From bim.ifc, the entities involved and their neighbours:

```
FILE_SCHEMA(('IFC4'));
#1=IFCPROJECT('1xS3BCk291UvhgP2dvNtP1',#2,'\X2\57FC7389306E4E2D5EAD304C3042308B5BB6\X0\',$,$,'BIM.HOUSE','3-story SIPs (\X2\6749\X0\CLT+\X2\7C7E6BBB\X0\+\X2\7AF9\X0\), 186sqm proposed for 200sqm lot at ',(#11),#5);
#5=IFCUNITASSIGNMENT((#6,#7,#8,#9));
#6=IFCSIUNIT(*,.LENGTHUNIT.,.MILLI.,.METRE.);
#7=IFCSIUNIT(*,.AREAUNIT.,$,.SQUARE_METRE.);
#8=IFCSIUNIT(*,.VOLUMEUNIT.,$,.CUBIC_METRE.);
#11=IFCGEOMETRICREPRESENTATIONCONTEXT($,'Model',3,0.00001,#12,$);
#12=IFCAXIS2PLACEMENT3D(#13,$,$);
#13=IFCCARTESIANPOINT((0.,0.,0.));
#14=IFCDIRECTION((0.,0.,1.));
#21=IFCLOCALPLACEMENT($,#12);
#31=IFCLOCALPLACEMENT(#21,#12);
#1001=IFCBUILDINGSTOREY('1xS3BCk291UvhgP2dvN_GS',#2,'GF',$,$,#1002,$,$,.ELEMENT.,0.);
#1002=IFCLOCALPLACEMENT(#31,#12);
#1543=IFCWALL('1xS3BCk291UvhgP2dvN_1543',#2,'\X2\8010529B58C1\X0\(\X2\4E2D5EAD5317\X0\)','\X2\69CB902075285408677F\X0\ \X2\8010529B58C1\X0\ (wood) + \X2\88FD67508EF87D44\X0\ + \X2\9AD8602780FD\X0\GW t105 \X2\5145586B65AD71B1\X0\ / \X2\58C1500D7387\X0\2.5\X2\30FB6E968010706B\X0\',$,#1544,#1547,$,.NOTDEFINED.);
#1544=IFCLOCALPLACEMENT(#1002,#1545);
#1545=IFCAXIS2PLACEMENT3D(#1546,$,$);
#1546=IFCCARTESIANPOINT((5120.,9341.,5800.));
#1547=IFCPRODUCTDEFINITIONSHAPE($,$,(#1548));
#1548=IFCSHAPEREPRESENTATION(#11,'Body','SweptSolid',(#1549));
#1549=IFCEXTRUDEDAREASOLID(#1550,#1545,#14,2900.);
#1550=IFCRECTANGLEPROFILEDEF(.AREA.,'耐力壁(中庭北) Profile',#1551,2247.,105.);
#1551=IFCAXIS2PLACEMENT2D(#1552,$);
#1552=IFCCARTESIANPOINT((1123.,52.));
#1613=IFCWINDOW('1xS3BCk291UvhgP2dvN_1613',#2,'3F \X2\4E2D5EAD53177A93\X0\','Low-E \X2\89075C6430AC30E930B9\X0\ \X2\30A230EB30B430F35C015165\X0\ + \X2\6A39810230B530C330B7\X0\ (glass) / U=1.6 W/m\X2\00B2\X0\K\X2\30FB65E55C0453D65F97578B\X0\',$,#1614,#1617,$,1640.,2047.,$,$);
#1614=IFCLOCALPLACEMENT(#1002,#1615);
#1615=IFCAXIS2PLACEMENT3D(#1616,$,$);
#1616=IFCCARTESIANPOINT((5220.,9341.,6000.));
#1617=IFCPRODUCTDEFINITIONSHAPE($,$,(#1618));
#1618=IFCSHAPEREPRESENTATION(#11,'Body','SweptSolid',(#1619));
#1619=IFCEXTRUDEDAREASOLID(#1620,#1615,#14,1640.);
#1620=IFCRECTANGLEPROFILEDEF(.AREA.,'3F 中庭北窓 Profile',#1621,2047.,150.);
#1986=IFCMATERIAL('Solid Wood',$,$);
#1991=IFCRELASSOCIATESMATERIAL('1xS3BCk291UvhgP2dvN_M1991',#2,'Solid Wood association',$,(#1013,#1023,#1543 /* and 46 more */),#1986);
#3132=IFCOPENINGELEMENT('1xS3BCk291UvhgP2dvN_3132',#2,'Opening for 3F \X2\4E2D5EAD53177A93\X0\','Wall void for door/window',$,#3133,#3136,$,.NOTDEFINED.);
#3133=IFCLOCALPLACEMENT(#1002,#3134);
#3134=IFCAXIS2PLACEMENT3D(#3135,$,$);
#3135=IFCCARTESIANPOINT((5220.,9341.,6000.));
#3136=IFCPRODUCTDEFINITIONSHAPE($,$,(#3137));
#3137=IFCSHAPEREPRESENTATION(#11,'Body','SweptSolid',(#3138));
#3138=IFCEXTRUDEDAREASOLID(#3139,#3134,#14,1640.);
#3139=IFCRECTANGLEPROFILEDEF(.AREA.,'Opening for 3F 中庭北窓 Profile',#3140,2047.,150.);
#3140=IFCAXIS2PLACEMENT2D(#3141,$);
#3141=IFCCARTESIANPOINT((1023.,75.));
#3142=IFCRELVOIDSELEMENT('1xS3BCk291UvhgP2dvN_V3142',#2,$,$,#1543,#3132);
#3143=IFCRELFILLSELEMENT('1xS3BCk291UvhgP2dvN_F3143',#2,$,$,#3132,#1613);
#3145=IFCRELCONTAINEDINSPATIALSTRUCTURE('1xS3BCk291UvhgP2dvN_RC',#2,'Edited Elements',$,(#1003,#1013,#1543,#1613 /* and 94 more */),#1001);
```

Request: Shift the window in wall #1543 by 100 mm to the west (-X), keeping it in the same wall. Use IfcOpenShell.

```python
import ifcopenshell
import ifcopenshell.api.geometry
import ifcopenshell.util.placement

model = ifcopenshell.open("bim.ifc")

window = model.by_guid("1xS3BCk291UvhgP2dvN_1613")
opening = window.FillsVoids[0].RelatingOpeningElement
wall = opening.VoidsElements[0].RelatingBuildingElement

wall_matrix = ifcopenshell.util.placement.get_local_placement(wall.ObjectPlacement)
shift = wall_matrix[:3, 0] * -100.0
before = ifcopenshell.util.placement.get_local_placement(window.ObjectPlacement)[:3, 3].copy()

# The window is not placed relative to its opening, so move both.
for product in (opening, window):
    matrix = ifcopenshell.util.placement.get_local_placement(product.ObjectPlacement)
    matrix[:3, 3] += shift
    ifcopenshell.api.geometry.edit_object_placement(model, product=product, matrix=matrix, is_si=False)

after = ifcopenshell.util.placement.get_local_placement(window.ObjectPlacement)[:3, 3]
print("window moved by", (after - before).round(3) + 0.0)

model.write("bim-out.ifc")
```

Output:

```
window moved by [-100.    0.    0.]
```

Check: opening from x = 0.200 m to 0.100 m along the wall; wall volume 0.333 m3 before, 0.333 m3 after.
